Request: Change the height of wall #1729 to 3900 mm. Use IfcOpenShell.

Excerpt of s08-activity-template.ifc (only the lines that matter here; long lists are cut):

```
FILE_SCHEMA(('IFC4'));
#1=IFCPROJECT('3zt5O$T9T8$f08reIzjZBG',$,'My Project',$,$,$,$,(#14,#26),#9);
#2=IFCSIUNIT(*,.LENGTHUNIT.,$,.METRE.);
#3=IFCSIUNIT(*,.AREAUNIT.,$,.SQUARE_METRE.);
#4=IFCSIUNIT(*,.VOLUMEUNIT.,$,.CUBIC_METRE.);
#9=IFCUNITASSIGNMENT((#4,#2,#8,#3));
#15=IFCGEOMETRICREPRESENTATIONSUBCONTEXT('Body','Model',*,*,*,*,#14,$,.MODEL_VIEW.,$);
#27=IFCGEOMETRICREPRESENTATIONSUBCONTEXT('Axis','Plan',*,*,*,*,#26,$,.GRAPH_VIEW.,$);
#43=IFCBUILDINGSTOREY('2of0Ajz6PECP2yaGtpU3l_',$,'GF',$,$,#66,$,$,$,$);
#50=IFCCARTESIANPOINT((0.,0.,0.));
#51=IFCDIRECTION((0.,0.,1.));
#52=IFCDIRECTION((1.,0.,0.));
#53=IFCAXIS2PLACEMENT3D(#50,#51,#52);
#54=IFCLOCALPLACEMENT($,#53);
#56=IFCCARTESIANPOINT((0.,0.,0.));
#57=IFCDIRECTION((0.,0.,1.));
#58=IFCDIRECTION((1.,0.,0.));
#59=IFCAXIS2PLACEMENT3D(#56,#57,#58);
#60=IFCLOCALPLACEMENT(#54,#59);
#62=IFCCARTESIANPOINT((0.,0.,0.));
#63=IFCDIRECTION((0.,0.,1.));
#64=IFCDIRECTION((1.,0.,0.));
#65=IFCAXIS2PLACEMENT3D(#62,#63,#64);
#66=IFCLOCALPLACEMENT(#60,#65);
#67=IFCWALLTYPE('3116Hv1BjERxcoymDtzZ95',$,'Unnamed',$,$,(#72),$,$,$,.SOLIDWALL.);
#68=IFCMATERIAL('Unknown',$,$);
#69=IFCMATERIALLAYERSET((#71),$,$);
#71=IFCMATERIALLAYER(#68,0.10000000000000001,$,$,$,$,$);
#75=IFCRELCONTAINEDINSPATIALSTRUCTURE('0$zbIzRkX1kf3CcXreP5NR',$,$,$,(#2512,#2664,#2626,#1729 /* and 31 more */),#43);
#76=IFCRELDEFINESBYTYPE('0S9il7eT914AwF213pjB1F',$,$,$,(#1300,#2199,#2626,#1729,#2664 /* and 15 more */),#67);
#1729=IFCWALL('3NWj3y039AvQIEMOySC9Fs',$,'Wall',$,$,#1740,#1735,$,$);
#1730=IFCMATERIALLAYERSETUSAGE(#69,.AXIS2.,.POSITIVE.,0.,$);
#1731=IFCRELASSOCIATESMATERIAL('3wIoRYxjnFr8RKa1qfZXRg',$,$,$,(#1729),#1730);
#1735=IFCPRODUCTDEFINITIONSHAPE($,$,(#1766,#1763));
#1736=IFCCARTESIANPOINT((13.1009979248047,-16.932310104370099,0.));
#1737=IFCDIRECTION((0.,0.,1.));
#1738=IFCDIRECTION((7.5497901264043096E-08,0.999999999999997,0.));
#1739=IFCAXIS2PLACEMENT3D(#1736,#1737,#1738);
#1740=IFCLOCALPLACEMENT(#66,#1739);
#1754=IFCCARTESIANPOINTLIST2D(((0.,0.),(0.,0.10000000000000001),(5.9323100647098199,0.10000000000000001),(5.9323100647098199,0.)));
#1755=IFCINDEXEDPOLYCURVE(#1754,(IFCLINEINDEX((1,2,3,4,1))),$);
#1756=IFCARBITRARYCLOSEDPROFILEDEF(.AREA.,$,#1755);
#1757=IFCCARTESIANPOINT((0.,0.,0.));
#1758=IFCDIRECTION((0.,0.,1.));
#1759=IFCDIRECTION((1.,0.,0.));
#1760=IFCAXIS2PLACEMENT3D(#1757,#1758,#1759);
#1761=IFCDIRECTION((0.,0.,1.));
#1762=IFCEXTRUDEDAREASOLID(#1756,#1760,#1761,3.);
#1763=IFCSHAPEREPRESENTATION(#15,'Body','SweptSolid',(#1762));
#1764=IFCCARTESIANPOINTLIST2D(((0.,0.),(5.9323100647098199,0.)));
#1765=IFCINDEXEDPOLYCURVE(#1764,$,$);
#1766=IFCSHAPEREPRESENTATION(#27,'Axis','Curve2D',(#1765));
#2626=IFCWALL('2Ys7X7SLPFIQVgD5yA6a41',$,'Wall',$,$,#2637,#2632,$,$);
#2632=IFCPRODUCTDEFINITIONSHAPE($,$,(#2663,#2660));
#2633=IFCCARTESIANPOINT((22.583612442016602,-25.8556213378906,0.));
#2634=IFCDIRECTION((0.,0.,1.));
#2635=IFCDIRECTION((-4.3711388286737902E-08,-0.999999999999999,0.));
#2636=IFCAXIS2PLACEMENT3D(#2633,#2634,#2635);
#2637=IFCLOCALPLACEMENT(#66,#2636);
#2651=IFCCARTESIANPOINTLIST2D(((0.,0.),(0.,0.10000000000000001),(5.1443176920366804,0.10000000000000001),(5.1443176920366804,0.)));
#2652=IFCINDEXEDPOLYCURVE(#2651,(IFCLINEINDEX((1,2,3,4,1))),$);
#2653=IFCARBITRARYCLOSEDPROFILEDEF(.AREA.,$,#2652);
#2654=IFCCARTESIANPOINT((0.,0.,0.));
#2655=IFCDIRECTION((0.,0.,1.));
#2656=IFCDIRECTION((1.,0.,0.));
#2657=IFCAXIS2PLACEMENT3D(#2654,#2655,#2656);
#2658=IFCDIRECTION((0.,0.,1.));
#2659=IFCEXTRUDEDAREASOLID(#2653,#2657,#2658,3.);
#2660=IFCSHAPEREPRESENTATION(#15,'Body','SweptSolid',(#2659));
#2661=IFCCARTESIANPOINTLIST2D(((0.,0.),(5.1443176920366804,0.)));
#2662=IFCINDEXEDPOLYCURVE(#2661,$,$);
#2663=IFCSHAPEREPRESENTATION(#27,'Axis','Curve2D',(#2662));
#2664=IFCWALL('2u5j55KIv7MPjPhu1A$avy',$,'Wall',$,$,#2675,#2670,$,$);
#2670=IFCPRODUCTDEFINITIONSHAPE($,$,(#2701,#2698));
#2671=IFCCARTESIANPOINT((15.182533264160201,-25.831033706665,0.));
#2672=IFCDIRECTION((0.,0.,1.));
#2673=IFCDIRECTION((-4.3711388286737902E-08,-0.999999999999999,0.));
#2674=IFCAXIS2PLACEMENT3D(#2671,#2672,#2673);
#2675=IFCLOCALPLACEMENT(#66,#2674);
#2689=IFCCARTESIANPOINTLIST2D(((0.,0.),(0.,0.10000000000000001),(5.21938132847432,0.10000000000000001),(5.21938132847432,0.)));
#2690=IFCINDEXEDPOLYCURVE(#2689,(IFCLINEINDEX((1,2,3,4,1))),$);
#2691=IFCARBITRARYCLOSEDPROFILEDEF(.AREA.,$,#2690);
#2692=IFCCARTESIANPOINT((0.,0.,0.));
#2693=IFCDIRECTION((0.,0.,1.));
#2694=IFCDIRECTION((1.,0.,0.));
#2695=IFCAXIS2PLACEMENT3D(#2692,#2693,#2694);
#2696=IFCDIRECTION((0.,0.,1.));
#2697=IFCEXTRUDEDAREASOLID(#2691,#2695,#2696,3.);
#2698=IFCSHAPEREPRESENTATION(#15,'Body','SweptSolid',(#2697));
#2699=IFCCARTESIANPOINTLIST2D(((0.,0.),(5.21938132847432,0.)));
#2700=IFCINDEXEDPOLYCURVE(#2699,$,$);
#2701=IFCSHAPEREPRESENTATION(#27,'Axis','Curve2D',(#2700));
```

```python
import ifcopenshell
import ifcopenshell.geom
import ifcopenshell.util.representation
import ifcopenshell.util.shape
import ifcopenshell.util.unit

model = ifcopenshell.open("s08-activity-template.ifc")
unit_scale = ifcopenshell.util.unit.calculate_unit_scale(model)
settings = ifcopenshell.geom.settings()


def volume(element):
    """Net volume in cubic metres, openings subtracted."""
    shape = ifcopenshell.geom.create_shape(settings, element)
    return ifcopenshell.util.shape.get_volume(shape.geometry)


wall = model.by_guid("3NWj3y039AvQIEMOySC9Fs")
before = volume(wall)

body = ifcopenshell.util.representation.get_representation(wall, "Model", "Body")
solid = body.Items[0]
old_height = solid.Depth
solid.Depth = 3.9 / unit_scale
after = volume(wall)

print(f"height {old_height:g} -> {solid.Depth:g}, volume {before:.3f} -> {after:.3f} m3")

model.write("s08-activity-template_edited.ifc")
```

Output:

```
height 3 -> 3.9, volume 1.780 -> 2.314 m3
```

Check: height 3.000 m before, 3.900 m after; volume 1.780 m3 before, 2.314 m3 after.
